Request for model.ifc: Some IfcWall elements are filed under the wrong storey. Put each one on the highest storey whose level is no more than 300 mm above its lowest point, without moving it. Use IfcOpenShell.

First a look at what the model holds.

```python
import ifcopenshell
import ifcopenshell.util.element
import ifcopenshell.util.placement

model = ifcopenshell.open("model.ifc")
print(model.schema)
for storey in model.by_type("IfcBuildingStorey"):
    level = ifcopenshell.util.placement.get_storey_elevation(storey)
    count = sum(e.is_a("IfcWall") for e in ifcopenshell.util.element.get_contained(storey))
    print(storey.id(), storey.Name, round(level, 3), count, sep=" | ")
```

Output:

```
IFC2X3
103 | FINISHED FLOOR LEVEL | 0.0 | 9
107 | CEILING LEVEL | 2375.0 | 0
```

```python
import ifcopenshell
import ifcopenshell.api.spatial
import ifcopenshell.geom
import ifcopenshell.util.element
import ifcopenshell.util.placement
import ifcopenshell.util.shape
import ifcopenshell.util.unit

model = ifcopenshell.open("model.ifc")
unit_scale = ifcopenshell.util.unit.calculate_unit_scale(model)
settings = ifcopenshell.geom.settings()

levels = sorted(
    ((ifcopenshell.util.placement.get_storey_elevation(s) * unit_scale, s) for s in model.by_type("IfcBuildingStorey")),
    key=lambda pair: pair[0],
)

for e in model.by_type("IfcWall"):
    current = e.ContainedInStructure[0].RelatingStructure if e.ContainedInStructure else None
    if current is None or not current.is_a("IfcBuildingStorey"):
        continue
    shape = ifcopenshell.geom.create_shape(settings, e)
    bottom = ifcopenshell.util.shape.get_shape_bottom_elevation(shape, shape.geometry)
    below = [s for level, s in levels if level <= bottom + 0.3]
    storey = below[-1] if below else levels[0][1]
    if storey != current:
        # assign_container keeps the world position.
        ifcopenshell.api.spatial.assign_container(model, products=[e], relating_structure=storey)
        print(e.id(), current.Name, "->", storey.Name)

model.write("model-out.ifc")
```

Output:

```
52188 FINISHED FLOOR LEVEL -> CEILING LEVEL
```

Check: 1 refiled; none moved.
